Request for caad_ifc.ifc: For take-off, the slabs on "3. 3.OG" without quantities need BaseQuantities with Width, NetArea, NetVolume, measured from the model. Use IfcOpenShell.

First a look at what the model holds.

```python
import ifcopenshell
import ifcopenshell.util.element
import ifcopenshell.util.unit

model = ifcopenshell.open("caad_ifc.ifc")
print(model.schema)
for unit_type in ("LENGTHUNIT", "AREAUNIT", "VOLUMEUNIT"):
    print(unit_type, ifcopenshell.util.unit.calculate_unit_scale(model, unit_type))
storey = next(s for s in model.by_type("IfcBuildingStorey") if s.Name == "3. 3.OG")
slabs = [e for e in ifcopenshell.util.element.get_decomposition(storey) if e.is_a("IfcSlab")]
for e in sorted(slabs, key=lambda e: e.id()):
    print(e.id(), e.is_a(), e.Name, list(ifcopenshell.util.element.get_psets(e, qtos_only=True)), sep=" | ")
```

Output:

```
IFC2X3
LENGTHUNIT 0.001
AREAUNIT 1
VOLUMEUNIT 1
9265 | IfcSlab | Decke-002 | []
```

```python
import ifcopenshell
import ifcopenshell.api.pset
import ifcopenshell.geom
import ifcopenshell.util.element
import ifcopenshell.util.shape
import ifcopenshell.util.unit

model = ifcopenshell.open("caad_ifc.ifc")
unit_scale = ifcopenshell.util.unit.calculate_unit_scale(model)
area_scale = ifcopenshell.util.unit.calculate_unit_scale(model, "AREAUNIT")
volume_scale = ifcopenshell.util.unit.calculate_unit_scale(model, "VOLUMEUNIT")
settings = ifcopenshell.geom.settings()

storey = next(s for s in model.by_type("IfcBuildingStorey") if s.Name == "3. 3.OG")
slabs = [e for e in ifcopenshell.util.element.get_decomposition(storey) if e.is_a("IfcSlab")]

for e in sorted(slabs, key=lambda e: e.id()):
    if ifcopenshell.util.element.get_psets(e, qtos_only=True, should_inherit=False):
        continue
    # Geometry comes back in metres, in the element's own axes.
    shape = ifcopenshell.geom.create_shape(settings, e)
    values = {
        "Width": ifcopenshell.util.shape.get_z(shape.geometry) / unit_scale,
        "NetArea": ifcopenshell.util.shape.get_footprint_area(shape.geometry) / area_scale,
        "NetVolume": ifcopenshell.util.shape.get_volume(shape.geometry) / volume_scale,
    }
    qto = ifcopenshell.api.pset.add_qto(model, product=e, name="BaseQuantities")
    ifcopenshell.api.pset.edit_qto(model, qto=qto, properties=values)
    print(e.id(), {k: round(v, 3) for k, v in values.items()})

model.write("caad_ifc_updated.ifc")
```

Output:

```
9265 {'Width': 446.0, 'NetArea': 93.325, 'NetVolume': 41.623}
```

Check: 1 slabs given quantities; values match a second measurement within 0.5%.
